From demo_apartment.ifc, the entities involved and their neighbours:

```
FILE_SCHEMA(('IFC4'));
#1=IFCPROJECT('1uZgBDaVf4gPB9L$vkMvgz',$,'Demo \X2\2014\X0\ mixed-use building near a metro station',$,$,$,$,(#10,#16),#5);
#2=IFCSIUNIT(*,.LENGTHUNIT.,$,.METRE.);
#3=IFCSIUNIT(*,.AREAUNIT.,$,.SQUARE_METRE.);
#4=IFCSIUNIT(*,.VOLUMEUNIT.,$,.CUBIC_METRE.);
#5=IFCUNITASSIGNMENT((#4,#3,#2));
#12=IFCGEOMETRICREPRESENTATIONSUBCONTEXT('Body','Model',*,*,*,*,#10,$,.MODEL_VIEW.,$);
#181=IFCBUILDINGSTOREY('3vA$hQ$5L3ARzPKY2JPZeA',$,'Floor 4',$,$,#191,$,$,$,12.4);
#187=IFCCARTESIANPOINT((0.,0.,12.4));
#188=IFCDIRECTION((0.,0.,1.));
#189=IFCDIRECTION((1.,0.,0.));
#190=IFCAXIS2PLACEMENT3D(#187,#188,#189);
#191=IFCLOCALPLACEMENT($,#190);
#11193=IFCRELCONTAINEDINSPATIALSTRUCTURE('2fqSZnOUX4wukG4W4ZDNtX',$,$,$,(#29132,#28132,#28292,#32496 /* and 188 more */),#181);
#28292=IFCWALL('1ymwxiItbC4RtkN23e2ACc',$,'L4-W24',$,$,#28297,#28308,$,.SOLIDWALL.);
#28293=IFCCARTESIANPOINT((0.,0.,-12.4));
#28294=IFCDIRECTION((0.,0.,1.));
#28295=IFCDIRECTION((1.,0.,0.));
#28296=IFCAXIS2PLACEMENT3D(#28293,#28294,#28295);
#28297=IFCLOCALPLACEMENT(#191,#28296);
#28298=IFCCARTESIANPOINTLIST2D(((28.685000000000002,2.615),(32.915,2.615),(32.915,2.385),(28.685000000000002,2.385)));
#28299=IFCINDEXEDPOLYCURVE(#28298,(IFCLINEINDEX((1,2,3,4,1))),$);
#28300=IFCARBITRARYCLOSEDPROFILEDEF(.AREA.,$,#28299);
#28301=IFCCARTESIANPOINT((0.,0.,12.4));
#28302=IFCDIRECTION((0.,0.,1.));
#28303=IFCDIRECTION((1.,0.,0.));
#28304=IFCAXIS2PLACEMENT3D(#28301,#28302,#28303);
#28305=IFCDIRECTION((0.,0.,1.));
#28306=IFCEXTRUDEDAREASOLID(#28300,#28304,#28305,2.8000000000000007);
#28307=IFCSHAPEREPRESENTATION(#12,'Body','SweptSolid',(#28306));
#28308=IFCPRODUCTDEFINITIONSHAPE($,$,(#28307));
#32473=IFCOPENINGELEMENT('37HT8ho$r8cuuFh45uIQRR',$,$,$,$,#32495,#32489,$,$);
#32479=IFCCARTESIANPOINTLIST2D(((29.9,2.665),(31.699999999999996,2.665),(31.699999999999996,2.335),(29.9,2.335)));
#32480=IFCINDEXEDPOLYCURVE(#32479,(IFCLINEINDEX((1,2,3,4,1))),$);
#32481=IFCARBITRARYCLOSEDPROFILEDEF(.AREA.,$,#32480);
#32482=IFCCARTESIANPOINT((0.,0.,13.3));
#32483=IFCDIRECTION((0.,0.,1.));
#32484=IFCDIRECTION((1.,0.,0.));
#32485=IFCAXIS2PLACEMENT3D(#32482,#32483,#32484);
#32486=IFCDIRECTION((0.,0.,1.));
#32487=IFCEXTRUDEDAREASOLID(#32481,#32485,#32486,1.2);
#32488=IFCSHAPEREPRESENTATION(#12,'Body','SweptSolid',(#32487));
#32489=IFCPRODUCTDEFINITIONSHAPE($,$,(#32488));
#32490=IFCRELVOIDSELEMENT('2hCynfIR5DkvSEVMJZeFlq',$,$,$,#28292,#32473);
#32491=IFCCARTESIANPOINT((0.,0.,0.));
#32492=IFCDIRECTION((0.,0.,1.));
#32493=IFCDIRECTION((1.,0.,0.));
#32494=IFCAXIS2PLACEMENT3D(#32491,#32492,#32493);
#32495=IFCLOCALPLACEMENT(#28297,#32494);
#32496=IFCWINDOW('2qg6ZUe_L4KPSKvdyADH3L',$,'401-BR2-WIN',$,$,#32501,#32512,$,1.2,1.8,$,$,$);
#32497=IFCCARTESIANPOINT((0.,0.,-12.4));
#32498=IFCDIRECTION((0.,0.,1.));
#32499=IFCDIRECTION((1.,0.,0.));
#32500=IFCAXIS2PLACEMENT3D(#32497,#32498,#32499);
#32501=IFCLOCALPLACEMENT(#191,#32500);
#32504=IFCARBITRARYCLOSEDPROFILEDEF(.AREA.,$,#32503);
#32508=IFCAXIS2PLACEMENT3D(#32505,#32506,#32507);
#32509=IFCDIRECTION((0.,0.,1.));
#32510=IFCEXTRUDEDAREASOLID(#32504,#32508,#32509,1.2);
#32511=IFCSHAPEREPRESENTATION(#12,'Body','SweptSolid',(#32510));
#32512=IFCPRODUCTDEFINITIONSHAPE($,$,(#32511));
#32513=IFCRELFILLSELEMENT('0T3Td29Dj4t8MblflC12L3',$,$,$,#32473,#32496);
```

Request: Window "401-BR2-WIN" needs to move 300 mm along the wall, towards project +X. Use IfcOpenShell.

```python
import ifcopenshell
import ifcopenshell.api.geometry
import ifcopenshell.util.placement
import ifcopenshell.util.unit

model = ifcopenshell.open("demo_apartment.ifc")
unit_scale = ifcopenshell.util.unit.calculate_unit_scale(model)

window = model.by_guid("2qg6ZUe_L4KPSKvdyADH3L")
opening = window.FillsVoids[0].RelatingOpeningElement
wall = opening.VoidsElements[0].RelatingBuildingElement

wall_matrix = ifcopenshell.util.placement.get_local_placement(wall.ObjectPlacement)
shift = wall_matrix[:3, 0] * 0.3 / unit_scale
before = ifcopenshell.util.placement.get_local_placement(window.ObjectPlacement)[:3, 3].copy()

# The window is not placed relative to its opening, so move both.
for product in (opening, window):
    matrix = ifcopenshell.util.placement.get_local_placement(product.ObjectPlacement)
    matrix[:3, 3] += shift
    ifcopenshell.api.geometry.edit_object_placement(model, product=product, matrix=matrix, is_si=False)

after = ifcopenshell.util.placement.get_local_placement(window.ObjectPlacement)[:3, 3]
print("window moved by", (after - before).round(3) + 0.0)

model.write("demo_apartment-out.ifc")
```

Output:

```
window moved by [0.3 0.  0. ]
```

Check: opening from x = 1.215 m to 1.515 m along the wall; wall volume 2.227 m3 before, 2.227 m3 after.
